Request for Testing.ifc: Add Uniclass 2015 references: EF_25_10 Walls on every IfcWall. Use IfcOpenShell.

First a look at what the model holds.

```python
import ifcopenshell

model = ifcopenshell.open("Testing.ifc")
print(model.schema)
print("classifications:", [c.Name for c in model.by_type("IfcClassification")])
for ifc_class in ("IfcDoor", "IfcRoof", "IfcStair", "IfcWall", "IfcWindow"):
    print(ifc_class, len(model.by_type(ifc_class)))
```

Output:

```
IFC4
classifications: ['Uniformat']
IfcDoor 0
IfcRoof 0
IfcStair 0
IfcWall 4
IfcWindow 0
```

```python
import ifcopenshell
import ifcopenshell.api.classification

model = ifcopenshell.open("Testing.ifc")

system = ifcopenshell.api.classification.add_classification(model, classification="Uniclass 2015")

codes = {
    "IfcWall": ("EF_25_10", "Walls"),
}
for ifc_class, (code, name) in codes.items():
    products = model.by_type(ifc_class)
    ifcopenshell.api.classification.add_reference(
        model, products=products, classification=system, identification=code, name=name
    )
    print(code, len(products))

model.write("Testing_edited.ifc")
```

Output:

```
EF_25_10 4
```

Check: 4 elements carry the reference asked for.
